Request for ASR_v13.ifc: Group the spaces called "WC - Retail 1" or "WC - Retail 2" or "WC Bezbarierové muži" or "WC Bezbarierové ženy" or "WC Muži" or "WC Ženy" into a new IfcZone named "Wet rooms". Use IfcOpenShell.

First a look at what the model holds.

```python
import ifcopenshell

model = ifcopenshell.open("ASR_v13.ifc")
print(model.schema)
seen = {}
for space in model.by_type("IfcSpace"):
    seen[space.LongName] = seen.get(space.LongName, 0) + 1
for name, count in sorted(seen.items(), key=str):
    print(count, "x", name)
print("zones:", [z.Name for z in model.by_type("IfcZone")][:20])
```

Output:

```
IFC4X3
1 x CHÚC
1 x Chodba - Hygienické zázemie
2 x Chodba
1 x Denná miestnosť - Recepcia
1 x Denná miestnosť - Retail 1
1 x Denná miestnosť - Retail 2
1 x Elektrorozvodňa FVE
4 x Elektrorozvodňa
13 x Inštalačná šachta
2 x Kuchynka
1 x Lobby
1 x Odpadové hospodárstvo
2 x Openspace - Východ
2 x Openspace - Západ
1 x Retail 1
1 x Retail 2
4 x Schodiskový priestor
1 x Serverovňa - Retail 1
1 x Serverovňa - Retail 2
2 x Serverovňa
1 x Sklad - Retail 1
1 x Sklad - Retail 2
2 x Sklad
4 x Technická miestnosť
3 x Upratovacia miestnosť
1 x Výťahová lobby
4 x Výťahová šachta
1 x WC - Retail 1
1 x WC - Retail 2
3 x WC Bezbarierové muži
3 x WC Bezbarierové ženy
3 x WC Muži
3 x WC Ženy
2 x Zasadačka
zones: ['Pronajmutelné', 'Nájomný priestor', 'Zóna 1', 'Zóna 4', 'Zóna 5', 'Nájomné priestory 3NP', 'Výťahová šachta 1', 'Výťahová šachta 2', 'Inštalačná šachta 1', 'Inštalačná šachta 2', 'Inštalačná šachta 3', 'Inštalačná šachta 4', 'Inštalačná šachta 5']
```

```python
import ifcopenshell
import ifcopenshell.api.group
import ifcopenshell.api.root

model = ifcopenshell.open("ASR_v13.ifc")

names = {"WC - Retail 1", "WC - Retail 2", "WC Bezbarierové muži", "WC Bezbarierové ženy", "WC Muži", "WC Ženy"}
spaces = [s for s in model.by_type("IfcSpace") if s.LongName in names]

zone = ifcopenshell.api.root.create_entity(model, ifc_class="IfcZone", name="Wet rooms")
ifcopenshell.api.group.assign_group(model, products=spaces, group=zone)
print(len(spaces), "spaces in", zone.Name)

model.write("ASR_v13_edited.ifc")
```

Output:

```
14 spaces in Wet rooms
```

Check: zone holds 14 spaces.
